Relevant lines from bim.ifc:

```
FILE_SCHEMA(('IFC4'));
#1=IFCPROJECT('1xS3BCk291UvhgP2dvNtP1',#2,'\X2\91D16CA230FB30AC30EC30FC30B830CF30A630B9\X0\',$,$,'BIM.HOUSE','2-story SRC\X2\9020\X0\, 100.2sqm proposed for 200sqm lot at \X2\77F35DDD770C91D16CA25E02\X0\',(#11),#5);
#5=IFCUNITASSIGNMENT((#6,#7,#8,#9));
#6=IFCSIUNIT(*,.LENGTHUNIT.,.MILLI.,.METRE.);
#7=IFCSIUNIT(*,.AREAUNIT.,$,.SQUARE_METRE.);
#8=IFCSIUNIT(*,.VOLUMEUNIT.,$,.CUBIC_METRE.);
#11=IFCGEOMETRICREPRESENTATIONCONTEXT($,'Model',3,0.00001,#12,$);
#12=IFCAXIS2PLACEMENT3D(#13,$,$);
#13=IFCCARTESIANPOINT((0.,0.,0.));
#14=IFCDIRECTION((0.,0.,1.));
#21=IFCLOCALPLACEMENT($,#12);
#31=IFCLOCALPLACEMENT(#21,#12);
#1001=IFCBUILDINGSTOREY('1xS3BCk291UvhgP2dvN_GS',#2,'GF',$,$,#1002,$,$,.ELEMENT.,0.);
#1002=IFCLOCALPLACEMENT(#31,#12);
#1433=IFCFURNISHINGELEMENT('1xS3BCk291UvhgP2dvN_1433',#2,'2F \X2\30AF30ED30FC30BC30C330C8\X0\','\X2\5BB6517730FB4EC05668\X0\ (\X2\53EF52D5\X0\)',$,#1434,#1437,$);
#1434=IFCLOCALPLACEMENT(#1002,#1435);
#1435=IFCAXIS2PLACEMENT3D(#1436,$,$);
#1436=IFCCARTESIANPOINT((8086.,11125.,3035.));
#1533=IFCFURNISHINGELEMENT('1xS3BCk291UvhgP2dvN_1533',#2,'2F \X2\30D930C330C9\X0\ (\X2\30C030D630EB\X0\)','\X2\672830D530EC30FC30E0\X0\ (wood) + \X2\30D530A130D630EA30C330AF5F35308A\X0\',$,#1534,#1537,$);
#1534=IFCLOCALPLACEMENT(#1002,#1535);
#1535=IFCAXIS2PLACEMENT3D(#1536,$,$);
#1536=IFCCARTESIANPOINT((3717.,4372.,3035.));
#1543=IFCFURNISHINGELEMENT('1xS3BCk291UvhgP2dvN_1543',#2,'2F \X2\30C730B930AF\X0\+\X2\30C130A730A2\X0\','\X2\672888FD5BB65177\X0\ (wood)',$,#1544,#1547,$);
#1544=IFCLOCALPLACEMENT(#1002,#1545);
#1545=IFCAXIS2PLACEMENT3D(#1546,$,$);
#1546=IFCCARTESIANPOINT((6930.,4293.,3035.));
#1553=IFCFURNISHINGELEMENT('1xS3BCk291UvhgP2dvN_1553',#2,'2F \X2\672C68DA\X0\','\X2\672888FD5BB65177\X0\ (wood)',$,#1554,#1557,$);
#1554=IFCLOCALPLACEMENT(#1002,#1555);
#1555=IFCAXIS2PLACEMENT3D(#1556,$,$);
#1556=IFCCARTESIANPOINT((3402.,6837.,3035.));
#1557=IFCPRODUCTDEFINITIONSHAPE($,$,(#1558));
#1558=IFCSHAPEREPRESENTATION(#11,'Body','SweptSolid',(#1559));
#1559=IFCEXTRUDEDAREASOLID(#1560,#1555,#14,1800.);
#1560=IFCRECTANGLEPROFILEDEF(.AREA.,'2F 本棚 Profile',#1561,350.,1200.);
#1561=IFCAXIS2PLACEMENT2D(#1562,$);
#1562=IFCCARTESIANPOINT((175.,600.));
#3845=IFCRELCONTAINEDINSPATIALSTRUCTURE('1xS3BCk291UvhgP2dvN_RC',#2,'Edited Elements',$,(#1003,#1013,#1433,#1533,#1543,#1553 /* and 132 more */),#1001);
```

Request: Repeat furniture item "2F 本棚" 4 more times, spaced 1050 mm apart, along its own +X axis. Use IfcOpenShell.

```python
import ifcopenshell
import ifcopenshell.api.geometry
import ifcopenshell.api.root
import ifcopenshell.util.element
import ifcopenshell.util.placement

model = ifcopenshell.open("bim.ifc")


def reuse_history(source, copy):
    """copy_class also copies each property set's owner history, people and application; keep the originals."""
    for rel in copy.IsDefinedBy:
        if rel.is_a("IfcRelDefinesByProperties") and (history := rel.RelatingPropertyDefinition.OwnerHistory):
            rel.RelatingPropertyDefinition.OwnerHistory = source.OwnerHistory
            ifcopenshell.util.element.remove_deep2(model, history)


source = model.by_guid("1xS3BCk291UvhgP2dvN_1553")
base = ifcopenshell.util.placement.get_local_placement(source.ObjectPlacement)
step = base[:3, 0] * 1050.0

for i in range(1, 5):
    copy = ifcopenshell.api.root.copy_class(model, product=source)
    copy.Representation = ifcopenshell.util.element.copy_deep(
        model, source.Representation, exclude=["IfcGeometricRepresentationContext", "IfcRepresentationMap"]
    )
    reuse_history(source, copy)
    matrix = base.copy()
    matrix[:3, 3] += i * step
    print("added at", matrix[:3, 3].round(3) + 0.0)
    ifcopenshell.api.geometry.edit_object_placement(model, product=copy, matrix=matrix, is_si=False)

model.write("bim_edited.ifc")
```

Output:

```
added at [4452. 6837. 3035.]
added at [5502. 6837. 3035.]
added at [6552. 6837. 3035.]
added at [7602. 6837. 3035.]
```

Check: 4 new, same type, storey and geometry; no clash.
